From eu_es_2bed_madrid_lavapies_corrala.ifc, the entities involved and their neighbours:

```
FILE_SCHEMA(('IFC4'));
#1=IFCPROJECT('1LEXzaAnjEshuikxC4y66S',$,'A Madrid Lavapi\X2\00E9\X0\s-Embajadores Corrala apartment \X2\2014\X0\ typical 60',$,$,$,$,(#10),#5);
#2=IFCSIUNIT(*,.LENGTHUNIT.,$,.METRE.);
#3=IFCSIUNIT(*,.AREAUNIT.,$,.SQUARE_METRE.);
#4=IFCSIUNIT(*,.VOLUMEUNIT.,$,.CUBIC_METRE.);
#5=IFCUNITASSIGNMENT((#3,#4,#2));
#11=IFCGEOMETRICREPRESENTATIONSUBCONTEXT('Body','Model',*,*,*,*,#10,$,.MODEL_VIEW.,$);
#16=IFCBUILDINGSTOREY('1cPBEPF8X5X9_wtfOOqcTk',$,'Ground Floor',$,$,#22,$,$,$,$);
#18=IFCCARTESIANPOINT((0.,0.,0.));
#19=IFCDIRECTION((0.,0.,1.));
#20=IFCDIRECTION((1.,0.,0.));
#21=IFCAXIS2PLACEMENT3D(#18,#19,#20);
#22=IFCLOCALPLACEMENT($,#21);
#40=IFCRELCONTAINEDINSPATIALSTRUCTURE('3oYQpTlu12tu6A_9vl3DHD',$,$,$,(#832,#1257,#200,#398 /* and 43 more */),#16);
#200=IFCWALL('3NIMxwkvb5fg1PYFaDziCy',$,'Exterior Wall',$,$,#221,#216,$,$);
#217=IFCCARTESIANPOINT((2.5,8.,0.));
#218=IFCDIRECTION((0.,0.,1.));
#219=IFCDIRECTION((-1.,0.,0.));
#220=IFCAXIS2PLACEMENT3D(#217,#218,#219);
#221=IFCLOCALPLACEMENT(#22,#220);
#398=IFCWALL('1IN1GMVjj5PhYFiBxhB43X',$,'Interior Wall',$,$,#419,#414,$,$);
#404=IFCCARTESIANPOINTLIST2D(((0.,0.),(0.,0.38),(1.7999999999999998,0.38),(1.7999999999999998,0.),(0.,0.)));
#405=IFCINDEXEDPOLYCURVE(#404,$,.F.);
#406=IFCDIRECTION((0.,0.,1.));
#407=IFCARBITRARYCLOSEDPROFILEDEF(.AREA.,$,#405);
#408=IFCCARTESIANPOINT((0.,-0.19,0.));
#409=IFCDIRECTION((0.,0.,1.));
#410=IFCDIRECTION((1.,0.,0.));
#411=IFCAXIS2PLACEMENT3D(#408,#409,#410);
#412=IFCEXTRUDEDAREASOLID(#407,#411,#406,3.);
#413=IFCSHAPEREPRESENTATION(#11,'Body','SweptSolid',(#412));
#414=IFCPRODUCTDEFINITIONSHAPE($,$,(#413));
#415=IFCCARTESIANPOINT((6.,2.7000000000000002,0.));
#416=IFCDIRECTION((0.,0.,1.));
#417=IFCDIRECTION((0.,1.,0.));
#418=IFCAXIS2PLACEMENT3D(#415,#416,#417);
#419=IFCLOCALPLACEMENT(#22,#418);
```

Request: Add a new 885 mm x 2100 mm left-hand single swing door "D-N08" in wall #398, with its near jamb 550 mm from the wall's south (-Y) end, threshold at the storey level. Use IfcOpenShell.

```python
import numpy as np
import ifcopenshell
import ifcopenshell.api.feature
import ifcopenshell.api.geometry
import ifcopenshell.api.root
import ifcopenshell.api.spatial
import ifcopenshell.geom
import ifcopenshell.util.element
import ifcopenshell.util.placement
import ifcopenshell.util.representation
import ifcopenshell.util.shape
import ifcopenshell.util.unit

model = ifcopenshell.open("eu_es_2bed_madrid_lavapies_corrala.ifc")
unit_scale = ifcopenshell.util.unit.calculate_unit_scale(model)
settings = ifcopenshell.geom.settings()


def volume(element):
    """Net volume in cubic metres, openings subtracted."""
    shape = ifcopenshell.geom.create_shape(settings, element)
    return ifcopenshell.util.shape.get_volume(shape.geometry)


wall = model.by_id(398)
storey = ifcopenshell.util.element.get_container(wall, ifc_class="IfcBuildingStorey")
context = ifcopenshell.util.representation.get_context(model, "Model", "Body", "MODEL_VIEW")
before = volume(wall)

width, height, from_end, sill = 0.885, 2.1, 0.55, 0.0  # metres

# The wall runs along its own X axis, and the end named is its -X end.
wall_shape = ifcopenshell.geom.create_shape(settings, wall)
x, y, z = ifcopenshell.util.shape.get_vertices(wall_shape.geometry).T
start = x.min() + from_end
face, thickness = float(y.min()), float(y.max() - y.min())
wall_matrix = ifcopenshell.util.placement.get_local_placement(wall.ObjectPlacement)
level = ifcopenshell.util.placement.get_local_placement(storey.ObjectPlacement)[2, 3]


def in_wall(x, y):
    """Placement at x, y metres in the wall's axes, at sill height."""
    matrix = wall_matrix.copy()
    matrix[:, 3] = wall_matrix @ np.array([x / unit_scale, y / unit_scale, 0.0, 1.0])
    matrix[2, 3] = level + sill / unit_scale
    return matrix


# Opening: a box that overshoots both wall faces by 50 mm.
opening = ifcopenshell.api.root.create_entity(model, ifc_class="IfcOpeningElement", predefined_type="OPENING")
box = ifcopenshell.api.geometry.add_wall_representation(
    model, context=context, length=width, height=height, thickness=thickness + 0.1
)
ifcopenshell.api.geometry.assign_representation(model, product=opening, representation=box)
ifcopenshell.api.geometry.edit_object_placement(model, product=opening, matrix=in_wall(start, face - 0.05), is_si=False)
ifcopenshell.api.feature.add_feature(model, feature=opening, element=wall)

door = ifcopenshell.api.root.create_entity(model, ifc_class="IfcDoor", name="D-N08", predefined_type="DOOR")
door.OverallWidth, door.OverallHeight = width / unit_scale, height / unit_scale
door.OperationType = "SINGLE_SWING_LEFT"
body = ifcopenshell.api.geometry.add_door_representation(
    model,
    context=context,
    overall_width=door.OverallWidth,
    overall_height=door.OverallHeight,
    operation_type="SINGLE_SWING_LEFT",
    lining_properties={"LiningDepth": thickness / unit_scale, "ThresholdDepth": thickness / unit_scale},
)
ifcopenshell.api.geometry.assign_representation(model, product=door, representation=body)
ifcopenshell.api.spatial.assign_container(model, products=[door], relating_structure=storey)
ifcopenshell.api.feature.add_filling(model, opening=opening, element=door)

# The lining spans the wall, so the door starts at the wall face.
ifcopenshell.api.geometry.edit_object_placement(model, product=door, matrix=in_wall(start, face), is_si=False)

after = volume(wall)

print(f"wall volume {before:.3f} -> {after:.3f} m3")

model.write("eu_es_2bed_madrid_lavapies_corrala_updated.ifc")
```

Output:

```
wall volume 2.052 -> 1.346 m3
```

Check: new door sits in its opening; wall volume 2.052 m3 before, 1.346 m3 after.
